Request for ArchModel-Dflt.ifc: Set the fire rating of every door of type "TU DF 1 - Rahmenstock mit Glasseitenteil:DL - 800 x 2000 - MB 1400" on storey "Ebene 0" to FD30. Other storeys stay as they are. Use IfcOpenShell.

First a look at what the model holds.

```python
import ifcopenshell
import ifcopenshell.util.element

model = ifcopenshell.open("ArchModel-Dflt.ifc")
print(model.schema)
storey = next(s for s in model.by_type("IfcBuildingStorey") if s.Name == "Ebene 0")
doors = [e for e in ifcopenshell.util.element.get_decomposition(storey) if e.is_a("IfcDoor")]
seen = {}
for e in doors:
    element_type = ifcopenshell.util.element.get_type(e)
    key = (element_type.Name if element_type != e and element_type else None, ifcopenshell.util.element.get_pset(e, "Pset_DoorCommon", "FireRating"))
    seen[key] = seen.get(key, 0) + 1
for (name, value), count in sorted(seen.items(), key=str):
    print(count, "x", name, "|", value)
```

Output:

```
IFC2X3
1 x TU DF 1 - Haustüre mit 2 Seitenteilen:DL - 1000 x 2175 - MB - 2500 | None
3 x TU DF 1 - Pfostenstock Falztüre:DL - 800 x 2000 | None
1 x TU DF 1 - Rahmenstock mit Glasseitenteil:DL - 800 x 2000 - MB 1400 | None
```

```python
import ifcopenshell
import ifcopenshell.api.pset
import ifcopenshell.util.element

model = ifcopenshell.open("ArchModel-Dflt.ifc")

storey = next(s for s in model.by_type("IfcBuildingStorey") if s.Name == "Ebene 0")
doors = [e for e in ifcopenshell.util.element.get_decomposition(storey) if e.is_a("IfcDoor")]

count = 0
for e in doors:
    element_type = ifcopenshell.util.element.get_type(e)
    if element_type in (None, e) or element_type.Name != "TU DF 1 - Rahmenstock mit Glasseitenteil:DL - 800 x 2000 - MB 1400":
        continue
    # add_pset returns the element's existing set when there is one.
    pset = ifcopenshell.api.pset.add_pset(model, product=e, name="Pset_DoorCommon")
    ifcopenshell.api.pset.edit_pset(model, pset=pset, properties={"FireRating": "FD30"})
    count += 1

print(count, "doors updated")

model.write("ArchModel-Dflt_updated.ifc")
```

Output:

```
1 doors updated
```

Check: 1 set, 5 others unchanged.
